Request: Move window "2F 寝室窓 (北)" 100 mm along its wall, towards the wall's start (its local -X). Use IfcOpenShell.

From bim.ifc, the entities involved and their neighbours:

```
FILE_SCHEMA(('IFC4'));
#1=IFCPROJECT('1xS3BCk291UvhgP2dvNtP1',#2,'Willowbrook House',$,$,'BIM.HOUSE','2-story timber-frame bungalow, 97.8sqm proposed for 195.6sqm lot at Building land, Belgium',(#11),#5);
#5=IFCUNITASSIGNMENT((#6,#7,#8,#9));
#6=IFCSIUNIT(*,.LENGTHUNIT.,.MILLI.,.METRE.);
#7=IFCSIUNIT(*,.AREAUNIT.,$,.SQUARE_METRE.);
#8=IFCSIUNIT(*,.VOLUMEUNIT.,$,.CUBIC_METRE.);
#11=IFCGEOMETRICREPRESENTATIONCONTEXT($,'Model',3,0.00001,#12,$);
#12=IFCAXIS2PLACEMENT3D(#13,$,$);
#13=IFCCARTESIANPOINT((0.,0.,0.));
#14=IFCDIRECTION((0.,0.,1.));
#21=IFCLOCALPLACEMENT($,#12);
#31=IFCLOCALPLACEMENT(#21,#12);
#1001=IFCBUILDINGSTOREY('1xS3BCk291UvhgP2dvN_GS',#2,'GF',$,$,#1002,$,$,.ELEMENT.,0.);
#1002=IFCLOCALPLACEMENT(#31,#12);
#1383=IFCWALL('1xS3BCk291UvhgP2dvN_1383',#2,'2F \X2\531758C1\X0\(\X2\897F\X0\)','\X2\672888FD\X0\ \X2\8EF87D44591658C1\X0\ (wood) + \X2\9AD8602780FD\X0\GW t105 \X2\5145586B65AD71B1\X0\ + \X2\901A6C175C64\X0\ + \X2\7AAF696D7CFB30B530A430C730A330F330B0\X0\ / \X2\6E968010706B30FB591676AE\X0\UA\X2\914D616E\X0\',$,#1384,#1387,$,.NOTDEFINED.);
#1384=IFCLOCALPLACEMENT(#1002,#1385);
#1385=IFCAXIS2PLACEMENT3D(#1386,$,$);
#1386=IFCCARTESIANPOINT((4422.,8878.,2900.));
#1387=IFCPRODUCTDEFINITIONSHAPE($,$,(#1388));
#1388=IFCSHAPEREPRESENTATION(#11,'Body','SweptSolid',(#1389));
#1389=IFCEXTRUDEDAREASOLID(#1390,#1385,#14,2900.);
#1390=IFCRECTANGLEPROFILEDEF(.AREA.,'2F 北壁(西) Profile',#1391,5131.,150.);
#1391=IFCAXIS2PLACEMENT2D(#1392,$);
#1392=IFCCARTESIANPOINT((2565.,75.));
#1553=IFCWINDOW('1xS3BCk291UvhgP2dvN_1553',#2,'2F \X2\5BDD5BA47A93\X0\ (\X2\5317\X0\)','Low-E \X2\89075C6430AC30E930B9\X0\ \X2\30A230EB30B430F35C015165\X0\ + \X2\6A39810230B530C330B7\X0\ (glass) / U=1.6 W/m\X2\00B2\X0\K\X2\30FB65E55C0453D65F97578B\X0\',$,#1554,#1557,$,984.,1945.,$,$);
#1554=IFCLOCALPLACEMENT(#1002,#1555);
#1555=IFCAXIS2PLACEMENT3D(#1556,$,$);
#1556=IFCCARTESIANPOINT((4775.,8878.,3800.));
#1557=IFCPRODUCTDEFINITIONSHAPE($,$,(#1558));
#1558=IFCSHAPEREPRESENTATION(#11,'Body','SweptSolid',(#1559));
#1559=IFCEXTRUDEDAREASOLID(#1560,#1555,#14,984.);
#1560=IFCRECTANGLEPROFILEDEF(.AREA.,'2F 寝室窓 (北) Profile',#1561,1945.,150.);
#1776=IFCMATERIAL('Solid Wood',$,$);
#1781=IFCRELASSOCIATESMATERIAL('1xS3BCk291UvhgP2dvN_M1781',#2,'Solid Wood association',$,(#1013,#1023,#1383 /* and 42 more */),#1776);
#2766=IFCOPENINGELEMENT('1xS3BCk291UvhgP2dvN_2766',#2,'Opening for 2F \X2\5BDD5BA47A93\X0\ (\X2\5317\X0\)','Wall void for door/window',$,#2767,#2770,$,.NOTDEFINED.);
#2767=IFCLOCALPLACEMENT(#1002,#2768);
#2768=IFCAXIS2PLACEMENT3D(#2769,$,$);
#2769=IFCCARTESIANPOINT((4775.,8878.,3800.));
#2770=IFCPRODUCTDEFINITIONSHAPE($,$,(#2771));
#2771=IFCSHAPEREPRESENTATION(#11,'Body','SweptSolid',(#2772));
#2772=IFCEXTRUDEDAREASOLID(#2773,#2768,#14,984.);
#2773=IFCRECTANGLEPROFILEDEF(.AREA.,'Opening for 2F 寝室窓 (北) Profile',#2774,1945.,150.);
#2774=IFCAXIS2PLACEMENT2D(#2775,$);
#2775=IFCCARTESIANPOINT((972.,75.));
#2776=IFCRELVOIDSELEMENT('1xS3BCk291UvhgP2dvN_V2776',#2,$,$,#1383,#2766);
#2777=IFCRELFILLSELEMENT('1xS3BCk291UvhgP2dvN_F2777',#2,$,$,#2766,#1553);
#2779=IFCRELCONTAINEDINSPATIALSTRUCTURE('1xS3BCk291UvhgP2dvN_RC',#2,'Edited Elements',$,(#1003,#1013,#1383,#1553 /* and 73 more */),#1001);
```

```python
import ifcopenshell
import ifcopenshell.api.geometry
import ifcopenshell.util.placement
import ifcopenshell.util.unit

model = ifcopenshell.open("bim.ifc")
unit_scale = ifcopenshell.util.unit.calculate_unit_scale(model)

window = model.by_guid("1xS3BCk291UvhgP2dvN_1553")
opening = window.FillsVoids[0].RelatingOpeningElement
wall = opening.VoidsElements[0].RelatingBuildingElement

wall_matrix = ifcopenshell.util.placement.get_local_placement(wall.ObjectPlacement)
shift = wall_matrix[:3, 0] * -0.1 / unit_scale
before = ifcopenshell.util.placement.get_local_placement(window.ObjectPlacement)[:3, 3].copy()

# The window is not placed relative to its opening, so move both.
for product in (opening, window):
    matrix = ifcopenshell.util.placement.get_local_placement(product.ObjectPlacement)
    matrix[:3, 3] += shift
    ifcopenshell.api.geometry.edit_object_placement(model, product=product, matrix=matrix, is_si=False)

after = ifcopenshell.util.placement.get_local_placement(window.ObjectPlacement)[:3, 3]
print("window moved by", (after - before).round(3) + 0.0)

model.write("bim-out.ifc")
```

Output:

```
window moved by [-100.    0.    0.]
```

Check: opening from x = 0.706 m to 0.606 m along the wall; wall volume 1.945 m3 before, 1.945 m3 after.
